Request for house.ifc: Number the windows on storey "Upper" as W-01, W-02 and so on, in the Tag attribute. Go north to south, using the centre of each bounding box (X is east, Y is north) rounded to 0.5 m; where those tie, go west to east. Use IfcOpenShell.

First a look at what the model holds.

```python
import ifcopenshell
import ifcopenshell.util.element
import ifcopenshell.util.placement

model = ifcopenshell.open("house.ifc")
print(model.schema)
storey = next(s for s in model.by_type("IfcBuildingStorey") if s.Name == "Upper")
windows = [e for e in ifcopenshell.util.element.get_decomposition(storey) if e.is_a("IfcWindow")]
for e in sorted(windows, key=lambda e: e.id()):
    origin = ifcopenshell.util.placement.get_local_placement(e.ObjectPlacement)[:3, 3]
    print(e.id(), e.Tag, e.Name, origin.round(2) + 0.0, sep=" | ")
```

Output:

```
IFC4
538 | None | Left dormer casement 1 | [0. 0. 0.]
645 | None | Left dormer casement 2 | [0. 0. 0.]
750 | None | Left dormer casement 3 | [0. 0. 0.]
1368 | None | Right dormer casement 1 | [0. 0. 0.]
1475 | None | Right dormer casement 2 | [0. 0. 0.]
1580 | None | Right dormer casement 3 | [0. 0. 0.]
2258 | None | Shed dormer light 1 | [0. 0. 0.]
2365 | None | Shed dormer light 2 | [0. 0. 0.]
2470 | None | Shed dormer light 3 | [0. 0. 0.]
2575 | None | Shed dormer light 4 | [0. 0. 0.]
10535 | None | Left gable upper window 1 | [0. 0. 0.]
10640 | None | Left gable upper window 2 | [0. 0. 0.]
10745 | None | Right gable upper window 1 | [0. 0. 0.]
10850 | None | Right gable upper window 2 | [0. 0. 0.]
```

```python
import ifcopenshell
import ifcopenshell.geom
import ifcopenshell.util.element
import ifcopenshell.util.shape

model = ifcopenshell.open("house.ifc")
settings = ifcopenshell.geom.settings()
settings.set("use-world-coords", True)


def centre(element):
    shape = ifcopenshell.geom.create_shape(settings, element)
    return ifcopenshell.util.shape.get_bbox_centroid(shape.geometry)


storey = next(s for s in model.by_type("IfcBuildingStorey") if s.Name == "Upper")
windows = [e for e in ifcopenshell.util.element.get_decomposition(storey) if e.is_a("IfcWindow")]

# Insertion points can sit at a corner or the storey origin, so sort by the geometry (in metres).
centres = {e: centre(e) for e in windows}
windows.sort(key=lambda e: (-round(centres[e][1] / 0.5), centres[e][0]))

for i, e in enumerate(windows, start=1):
    number = f"W-{i:02d}"
    e.Tag = number
    print(e.id(), number)

model.write("house_v2.ifc")
```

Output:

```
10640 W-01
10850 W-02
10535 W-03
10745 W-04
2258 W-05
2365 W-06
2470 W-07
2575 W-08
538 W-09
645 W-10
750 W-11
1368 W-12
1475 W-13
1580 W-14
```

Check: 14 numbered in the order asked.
